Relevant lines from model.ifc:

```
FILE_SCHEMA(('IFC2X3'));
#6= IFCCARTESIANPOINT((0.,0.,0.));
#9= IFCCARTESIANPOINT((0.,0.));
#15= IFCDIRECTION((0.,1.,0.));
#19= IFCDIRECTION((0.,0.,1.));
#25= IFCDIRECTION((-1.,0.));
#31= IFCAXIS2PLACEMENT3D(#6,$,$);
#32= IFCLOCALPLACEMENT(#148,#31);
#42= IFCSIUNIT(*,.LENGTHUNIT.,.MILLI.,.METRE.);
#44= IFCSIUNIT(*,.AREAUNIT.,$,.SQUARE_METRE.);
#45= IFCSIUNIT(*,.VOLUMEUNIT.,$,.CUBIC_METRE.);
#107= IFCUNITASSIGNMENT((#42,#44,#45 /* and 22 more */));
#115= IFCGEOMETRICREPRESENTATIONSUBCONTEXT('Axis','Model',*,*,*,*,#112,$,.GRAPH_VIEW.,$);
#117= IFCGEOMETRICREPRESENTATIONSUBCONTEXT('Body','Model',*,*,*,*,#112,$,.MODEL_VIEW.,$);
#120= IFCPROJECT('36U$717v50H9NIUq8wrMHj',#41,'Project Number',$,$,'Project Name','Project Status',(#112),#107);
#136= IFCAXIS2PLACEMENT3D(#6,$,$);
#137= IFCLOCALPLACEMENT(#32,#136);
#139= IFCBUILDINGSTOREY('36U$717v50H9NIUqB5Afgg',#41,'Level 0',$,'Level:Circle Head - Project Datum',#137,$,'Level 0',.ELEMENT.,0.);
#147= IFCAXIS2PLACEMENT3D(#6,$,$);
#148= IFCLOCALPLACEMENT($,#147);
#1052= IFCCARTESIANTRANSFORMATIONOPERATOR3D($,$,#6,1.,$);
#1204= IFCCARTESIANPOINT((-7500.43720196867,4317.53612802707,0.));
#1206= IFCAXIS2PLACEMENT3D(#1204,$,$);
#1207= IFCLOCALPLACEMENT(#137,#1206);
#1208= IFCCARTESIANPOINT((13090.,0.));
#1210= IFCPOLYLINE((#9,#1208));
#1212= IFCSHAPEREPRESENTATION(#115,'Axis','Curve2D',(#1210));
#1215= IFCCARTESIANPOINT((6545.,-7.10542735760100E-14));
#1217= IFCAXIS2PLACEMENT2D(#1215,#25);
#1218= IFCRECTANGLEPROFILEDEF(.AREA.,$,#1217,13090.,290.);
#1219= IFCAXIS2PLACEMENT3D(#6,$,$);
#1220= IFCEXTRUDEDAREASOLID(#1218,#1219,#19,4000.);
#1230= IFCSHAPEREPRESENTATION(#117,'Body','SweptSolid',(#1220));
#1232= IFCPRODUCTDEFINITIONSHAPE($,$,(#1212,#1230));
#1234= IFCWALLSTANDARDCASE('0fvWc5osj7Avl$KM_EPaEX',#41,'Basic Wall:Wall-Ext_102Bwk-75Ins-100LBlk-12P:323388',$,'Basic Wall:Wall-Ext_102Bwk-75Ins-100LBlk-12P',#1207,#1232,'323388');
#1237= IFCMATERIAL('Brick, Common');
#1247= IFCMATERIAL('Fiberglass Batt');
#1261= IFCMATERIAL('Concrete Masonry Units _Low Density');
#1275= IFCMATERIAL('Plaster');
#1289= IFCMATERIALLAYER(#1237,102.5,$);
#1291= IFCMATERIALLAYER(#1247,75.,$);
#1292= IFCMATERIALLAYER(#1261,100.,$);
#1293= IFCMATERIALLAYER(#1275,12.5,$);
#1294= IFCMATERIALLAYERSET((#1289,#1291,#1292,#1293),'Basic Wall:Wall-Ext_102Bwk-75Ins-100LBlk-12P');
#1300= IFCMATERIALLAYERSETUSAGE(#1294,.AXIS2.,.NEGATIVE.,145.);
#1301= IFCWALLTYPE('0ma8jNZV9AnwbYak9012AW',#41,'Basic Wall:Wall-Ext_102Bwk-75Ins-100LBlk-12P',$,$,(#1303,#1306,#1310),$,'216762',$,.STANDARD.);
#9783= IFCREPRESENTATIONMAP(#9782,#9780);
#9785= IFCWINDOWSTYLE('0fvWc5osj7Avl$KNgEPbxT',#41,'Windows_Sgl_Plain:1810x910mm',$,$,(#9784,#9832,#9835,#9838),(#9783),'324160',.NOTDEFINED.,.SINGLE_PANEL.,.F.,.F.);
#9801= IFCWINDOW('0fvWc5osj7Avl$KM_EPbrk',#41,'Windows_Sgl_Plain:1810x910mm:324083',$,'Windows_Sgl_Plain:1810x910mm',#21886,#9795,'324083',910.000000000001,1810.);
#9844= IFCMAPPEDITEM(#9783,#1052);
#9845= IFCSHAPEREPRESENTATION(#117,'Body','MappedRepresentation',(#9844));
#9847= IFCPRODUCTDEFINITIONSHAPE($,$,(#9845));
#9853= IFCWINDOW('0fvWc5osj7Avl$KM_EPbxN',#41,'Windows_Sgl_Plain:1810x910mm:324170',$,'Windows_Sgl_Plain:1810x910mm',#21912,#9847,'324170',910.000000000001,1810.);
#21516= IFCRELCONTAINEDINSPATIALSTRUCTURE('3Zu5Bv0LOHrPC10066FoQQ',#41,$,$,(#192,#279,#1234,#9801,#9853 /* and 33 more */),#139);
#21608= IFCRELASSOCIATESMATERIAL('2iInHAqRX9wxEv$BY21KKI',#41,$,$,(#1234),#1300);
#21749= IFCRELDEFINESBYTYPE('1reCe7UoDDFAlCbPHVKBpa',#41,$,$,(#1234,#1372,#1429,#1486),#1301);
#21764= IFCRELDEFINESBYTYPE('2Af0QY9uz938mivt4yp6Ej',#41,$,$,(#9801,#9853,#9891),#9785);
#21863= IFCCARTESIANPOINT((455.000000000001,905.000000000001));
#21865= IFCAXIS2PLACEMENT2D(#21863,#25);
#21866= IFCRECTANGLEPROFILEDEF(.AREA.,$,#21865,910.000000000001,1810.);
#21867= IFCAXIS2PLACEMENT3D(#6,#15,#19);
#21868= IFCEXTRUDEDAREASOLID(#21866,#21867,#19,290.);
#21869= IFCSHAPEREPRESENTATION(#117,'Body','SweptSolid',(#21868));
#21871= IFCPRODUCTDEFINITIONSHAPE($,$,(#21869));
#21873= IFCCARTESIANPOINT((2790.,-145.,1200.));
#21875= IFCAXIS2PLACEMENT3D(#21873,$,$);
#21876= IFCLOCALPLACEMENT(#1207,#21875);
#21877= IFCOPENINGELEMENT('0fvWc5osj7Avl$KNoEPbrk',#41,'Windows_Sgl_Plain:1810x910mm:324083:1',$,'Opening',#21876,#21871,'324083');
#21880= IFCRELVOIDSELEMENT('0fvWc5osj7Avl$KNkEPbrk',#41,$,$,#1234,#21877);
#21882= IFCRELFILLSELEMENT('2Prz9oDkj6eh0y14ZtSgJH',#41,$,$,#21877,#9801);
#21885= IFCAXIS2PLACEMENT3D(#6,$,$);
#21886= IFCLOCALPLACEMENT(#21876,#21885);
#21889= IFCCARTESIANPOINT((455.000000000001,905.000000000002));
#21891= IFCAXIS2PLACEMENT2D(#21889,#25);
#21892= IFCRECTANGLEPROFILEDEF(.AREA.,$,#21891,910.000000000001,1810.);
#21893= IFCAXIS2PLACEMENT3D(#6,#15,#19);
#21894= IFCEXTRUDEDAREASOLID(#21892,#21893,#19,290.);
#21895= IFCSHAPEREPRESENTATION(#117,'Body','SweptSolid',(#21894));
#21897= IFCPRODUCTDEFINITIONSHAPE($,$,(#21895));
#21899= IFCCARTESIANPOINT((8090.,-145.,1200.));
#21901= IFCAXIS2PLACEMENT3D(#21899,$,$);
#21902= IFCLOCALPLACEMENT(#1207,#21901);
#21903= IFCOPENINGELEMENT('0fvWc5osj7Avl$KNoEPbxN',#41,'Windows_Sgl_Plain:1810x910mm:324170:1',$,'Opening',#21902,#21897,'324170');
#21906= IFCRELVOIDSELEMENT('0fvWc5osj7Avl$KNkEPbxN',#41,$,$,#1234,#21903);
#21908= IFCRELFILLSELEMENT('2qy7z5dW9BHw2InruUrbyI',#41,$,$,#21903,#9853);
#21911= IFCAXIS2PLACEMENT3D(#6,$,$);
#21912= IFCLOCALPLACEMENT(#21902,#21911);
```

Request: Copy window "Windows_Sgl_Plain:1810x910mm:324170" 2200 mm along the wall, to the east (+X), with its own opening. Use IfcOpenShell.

```python
import ifcopenshell
import ifcopenshell.api.feature
import ifcopenshell.api.geometry
import ifcopenshell.api.root
import ifcopenshell.geom
import ifcopenshell.util.element
import ifcopenshell.util.placement
import ifcopenshell.util.shape
import ifcopenshell.util.unit

model = ifcopenshell.open("model.ifc")
unit_scale = ifcopenshell.util.unit.calculate_unit_scale(model)
settings = ifcopenshell.geom.settings()


def volume(element):
    """Net volume in cubic metres, openings subtracted."""
    shape = ifcopenshell.geom.create_shape(settings, element)
    return ifcopenshell.util.shape.get_volume(shape.geometry)


def reuse_history(source, copy):
    """copy_class also copies each property set's owner history, people and application; keep the originals."""
    for rel in copy.IsDefinedBy:
        if rel.is_a("IfcRelDefinesByProperties") and (history := rel.RelatingPropertyDefinition.OwnerHistory):
            rel.RelatingPropertyDefinition.OwnerHistory = source.OwnerHistory
            ifcopenshell.util.element.remove_deep2(model, history)


window = model.by_guid("0fvWc5osj7Avl$KM_EPbxN")
opening = window.FillsVoids[0].RelatingOpeningElement
wall = opening.VoidsElements[0].RelatingBuildingElement
before = volume(wall)
shift = ifcopenshell.util.placement.get_local_placement(wall.ObjectPlacement)[:3, 0] * 2.2 / unit_scale

# copy_class copies the void relationship, type, container and properties, but no geometry.
new_opening = ifcopenshell.api.root.copy_class(model, product=opening)
new_opening.Representation = ifcopenshell.util.element.copy_deep(
    model, opening.Representation, exclude=["IfcGeometricRepresentationContext", "IfcRepresentationMap"]
)
new_opening.Name = "Windows_Sgl_Plain:1810x910mm"
new_opening.Tag = None
new_window = ifcopenshell.api.root.copy_class(model, product=window)
new_window.Representation = ifcopenshell.util.element.copy_deep(
    model, window.Representation, exclude=["IfcGeometricRepresentationContext", "IfcRepresentationMap"]
)
new_window.Name = "Windows_Sgl_Plain:1810x910mm"
new_window.Tag = None
reuse_history(window, new_window)
fills = ifcopenshell.api.feature.add_filling(model, opening=new_opening, element=new_window)
fills.OwnerHistory = new_window.OwnerHistory  # required in IFC2X3

for old, new in ((opening, new_opening), (window, new_window)):
    matrix = ifcopenshell.util.placement.get_local_placement(old.ObjectPlacement)
    matrix[:3, 3] += shift
    ifcopenshell.api.geometry.edit_object_placement(model, product=new, matrix=matrix, is_si=False)

after = volume(wall)

print(f"wall volume {before:.3f} -> {after:.3f} m3")

model.write("model-out.ifc")
```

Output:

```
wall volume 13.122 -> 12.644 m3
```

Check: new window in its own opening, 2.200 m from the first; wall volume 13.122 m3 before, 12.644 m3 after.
